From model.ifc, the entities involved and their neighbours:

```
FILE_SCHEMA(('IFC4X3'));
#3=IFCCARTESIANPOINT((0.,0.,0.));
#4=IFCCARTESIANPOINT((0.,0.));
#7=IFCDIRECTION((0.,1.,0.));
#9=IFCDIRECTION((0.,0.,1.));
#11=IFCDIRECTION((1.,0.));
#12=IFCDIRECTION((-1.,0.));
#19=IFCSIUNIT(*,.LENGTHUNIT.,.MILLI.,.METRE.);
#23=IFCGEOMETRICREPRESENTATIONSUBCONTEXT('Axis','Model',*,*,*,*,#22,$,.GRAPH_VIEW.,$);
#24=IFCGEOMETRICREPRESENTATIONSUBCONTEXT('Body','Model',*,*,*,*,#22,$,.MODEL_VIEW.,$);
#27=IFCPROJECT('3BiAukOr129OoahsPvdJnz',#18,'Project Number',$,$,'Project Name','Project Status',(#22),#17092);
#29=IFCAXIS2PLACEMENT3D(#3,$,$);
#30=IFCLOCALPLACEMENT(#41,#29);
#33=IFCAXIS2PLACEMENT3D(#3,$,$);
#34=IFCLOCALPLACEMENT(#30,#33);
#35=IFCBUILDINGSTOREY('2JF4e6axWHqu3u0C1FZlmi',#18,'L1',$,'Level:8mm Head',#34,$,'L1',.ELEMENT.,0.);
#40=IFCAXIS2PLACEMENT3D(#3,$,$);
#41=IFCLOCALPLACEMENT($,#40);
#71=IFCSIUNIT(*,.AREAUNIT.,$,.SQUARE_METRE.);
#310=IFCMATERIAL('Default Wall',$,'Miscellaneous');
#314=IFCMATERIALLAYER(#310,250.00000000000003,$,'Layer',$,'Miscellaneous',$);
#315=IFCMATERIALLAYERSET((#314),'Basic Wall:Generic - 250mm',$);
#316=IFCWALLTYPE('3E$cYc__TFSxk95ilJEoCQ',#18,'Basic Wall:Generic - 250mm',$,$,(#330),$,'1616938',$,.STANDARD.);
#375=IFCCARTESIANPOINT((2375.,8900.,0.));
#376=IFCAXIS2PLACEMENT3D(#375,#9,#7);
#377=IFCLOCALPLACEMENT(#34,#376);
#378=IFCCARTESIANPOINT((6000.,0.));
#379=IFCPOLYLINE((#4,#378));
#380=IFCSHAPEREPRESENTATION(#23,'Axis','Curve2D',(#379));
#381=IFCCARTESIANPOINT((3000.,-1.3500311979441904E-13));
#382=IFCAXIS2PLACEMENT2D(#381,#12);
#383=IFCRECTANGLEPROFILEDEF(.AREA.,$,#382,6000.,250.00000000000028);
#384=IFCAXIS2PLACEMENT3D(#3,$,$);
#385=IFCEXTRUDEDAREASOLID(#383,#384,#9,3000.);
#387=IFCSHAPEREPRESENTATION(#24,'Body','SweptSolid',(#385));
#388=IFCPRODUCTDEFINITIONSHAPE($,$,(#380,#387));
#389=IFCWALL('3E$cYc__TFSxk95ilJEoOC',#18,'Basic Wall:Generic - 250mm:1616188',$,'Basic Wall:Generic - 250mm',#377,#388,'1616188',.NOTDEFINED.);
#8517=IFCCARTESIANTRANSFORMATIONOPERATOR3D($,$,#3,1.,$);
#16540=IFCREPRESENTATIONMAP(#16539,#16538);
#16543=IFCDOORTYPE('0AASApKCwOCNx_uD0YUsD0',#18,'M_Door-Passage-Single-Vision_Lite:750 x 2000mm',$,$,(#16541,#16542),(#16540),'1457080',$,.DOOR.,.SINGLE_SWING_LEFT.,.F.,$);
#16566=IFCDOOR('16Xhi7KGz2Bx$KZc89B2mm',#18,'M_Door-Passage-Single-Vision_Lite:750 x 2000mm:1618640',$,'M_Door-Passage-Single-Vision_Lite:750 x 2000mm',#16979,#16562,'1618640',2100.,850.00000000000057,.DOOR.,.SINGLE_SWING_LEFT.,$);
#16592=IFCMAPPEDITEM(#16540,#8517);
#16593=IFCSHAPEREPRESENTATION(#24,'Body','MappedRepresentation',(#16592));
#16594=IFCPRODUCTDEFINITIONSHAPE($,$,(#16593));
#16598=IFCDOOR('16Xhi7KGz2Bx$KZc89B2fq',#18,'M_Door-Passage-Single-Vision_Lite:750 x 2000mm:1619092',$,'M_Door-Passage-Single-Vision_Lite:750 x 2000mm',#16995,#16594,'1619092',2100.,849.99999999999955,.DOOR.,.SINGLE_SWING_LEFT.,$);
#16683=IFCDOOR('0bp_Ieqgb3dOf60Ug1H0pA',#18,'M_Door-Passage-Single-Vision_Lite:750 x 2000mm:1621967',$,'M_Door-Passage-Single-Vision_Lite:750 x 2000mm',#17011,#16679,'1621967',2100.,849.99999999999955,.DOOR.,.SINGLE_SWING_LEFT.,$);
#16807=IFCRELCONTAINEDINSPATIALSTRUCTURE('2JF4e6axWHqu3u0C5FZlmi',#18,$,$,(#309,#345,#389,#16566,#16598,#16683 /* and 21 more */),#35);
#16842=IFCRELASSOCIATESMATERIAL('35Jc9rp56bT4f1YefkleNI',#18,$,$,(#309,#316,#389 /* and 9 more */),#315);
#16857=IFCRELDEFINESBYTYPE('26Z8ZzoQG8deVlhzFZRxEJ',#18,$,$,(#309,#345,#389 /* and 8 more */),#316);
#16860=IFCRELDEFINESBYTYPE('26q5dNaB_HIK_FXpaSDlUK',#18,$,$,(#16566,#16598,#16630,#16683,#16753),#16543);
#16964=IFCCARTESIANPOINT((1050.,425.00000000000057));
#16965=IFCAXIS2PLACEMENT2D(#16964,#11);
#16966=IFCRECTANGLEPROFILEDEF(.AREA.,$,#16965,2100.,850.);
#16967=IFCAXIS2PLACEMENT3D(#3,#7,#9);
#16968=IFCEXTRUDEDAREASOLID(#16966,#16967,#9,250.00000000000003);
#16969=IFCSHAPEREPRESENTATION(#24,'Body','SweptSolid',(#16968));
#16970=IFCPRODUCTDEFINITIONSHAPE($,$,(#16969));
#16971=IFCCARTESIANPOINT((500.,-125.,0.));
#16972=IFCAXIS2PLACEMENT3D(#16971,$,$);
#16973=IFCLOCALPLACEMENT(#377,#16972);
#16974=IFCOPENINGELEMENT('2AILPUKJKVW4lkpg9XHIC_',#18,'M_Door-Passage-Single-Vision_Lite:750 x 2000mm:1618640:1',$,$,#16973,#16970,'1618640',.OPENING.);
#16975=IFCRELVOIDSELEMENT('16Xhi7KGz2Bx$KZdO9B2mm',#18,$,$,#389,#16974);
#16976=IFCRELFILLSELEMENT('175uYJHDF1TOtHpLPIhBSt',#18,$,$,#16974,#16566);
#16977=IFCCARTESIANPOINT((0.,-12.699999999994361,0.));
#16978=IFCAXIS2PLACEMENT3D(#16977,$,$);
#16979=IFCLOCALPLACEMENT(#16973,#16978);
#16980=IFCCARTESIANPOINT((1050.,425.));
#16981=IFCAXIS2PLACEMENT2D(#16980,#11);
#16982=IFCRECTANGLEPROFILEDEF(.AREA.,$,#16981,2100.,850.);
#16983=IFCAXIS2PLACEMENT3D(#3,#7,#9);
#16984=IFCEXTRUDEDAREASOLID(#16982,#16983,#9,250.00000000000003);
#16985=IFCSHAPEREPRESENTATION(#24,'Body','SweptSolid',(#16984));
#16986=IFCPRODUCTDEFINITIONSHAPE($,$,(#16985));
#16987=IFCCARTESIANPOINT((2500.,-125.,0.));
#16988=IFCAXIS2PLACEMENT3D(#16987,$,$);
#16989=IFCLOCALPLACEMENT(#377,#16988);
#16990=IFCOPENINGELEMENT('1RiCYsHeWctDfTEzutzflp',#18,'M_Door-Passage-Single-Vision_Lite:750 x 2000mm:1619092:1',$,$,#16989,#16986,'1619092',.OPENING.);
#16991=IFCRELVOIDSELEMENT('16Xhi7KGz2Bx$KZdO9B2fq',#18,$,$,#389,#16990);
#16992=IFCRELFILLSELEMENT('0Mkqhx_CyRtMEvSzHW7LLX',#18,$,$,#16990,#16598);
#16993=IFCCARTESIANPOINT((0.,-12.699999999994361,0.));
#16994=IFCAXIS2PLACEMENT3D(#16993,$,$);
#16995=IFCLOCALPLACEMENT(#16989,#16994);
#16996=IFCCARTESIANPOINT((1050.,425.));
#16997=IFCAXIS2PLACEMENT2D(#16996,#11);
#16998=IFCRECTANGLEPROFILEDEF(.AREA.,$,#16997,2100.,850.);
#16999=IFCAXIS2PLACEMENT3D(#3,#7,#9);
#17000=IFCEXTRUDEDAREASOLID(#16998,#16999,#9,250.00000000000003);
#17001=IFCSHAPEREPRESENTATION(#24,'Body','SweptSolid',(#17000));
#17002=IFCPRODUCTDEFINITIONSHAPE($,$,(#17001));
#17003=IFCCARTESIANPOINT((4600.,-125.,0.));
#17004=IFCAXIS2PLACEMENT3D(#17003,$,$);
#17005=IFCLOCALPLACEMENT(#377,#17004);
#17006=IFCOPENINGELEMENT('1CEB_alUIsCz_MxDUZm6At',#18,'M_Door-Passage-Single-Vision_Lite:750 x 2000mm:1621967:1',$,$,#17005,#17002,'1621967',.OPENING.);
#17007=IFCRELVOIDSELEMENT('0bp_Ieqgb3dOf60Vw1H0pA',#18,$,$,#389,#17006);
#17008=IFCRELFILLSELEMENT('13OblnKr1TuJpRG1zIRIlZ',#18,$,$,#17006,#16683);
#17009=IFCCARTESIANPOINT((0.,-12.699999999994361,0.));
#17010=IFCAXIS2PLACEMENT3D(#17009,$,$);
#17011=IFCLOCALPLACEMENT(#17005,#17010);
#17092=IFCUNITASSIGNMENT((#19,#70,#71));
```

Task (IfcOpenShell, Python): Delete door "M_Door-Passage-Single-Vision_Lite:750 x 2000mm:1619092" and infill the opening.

```python
import ifcopenshell
import ifcopenshell.api.feature
import ifcopenshell.api.root
import ifcopenshell.geom
import ifcopenshell.util.shape

model = ifcopenshell.open("model.ifc")
settings = ifcopenshell.geom.settings()


def volume(element):
    """Net volume in cubic metres, openings subtracted."""
    shape = ifcopenshell.geom.create_shape(settings, element)
    return ifcopenshell.util.shape.get_volume(shape.geometry)


door = model.by_id(16598)
opening = door.FillsVoids[0].RelatingOpeningElement
wall = opening.VoidsElements[0].RelatingBuildingElement
before = volume(wall)

ifcopenshell.api.root.remove_product(model, product=door)
ifcopenshell.api.feature.remove_feature(model, feature=opening)

after = volume(wall)

print(f"wall volume {before:.3f} -> {after:.3f} m3")

model.write("model-out.ifc")
```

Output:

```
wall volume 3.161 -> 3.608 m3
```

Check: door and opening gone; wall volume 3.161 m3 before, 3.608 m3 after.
